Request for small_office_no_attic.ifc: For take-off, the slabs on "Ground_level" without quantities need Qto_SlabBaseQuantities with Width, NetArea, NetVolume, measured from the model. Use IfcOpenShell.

First a look at what the model holds.

```python
import ifcopenshell
import ifcopenshell.util.element
import ifcopenshell.util.unit

model = ifcopenshell.open("small_office_no_attic.ifc")
print(model.schema)
for unit_type in ("LENGTHUNIT", "AREAUNIT", "VOLUMEUNIT"):
    print(unit_type, ifcopenshell.util.unit.calculate_unit_scale(model, unit_type))
storey = next(s for s in model.by_type("IfcBuildingStorey") if s.Name == "Ground_level")
slabs = [e for e in ifcopenshell.util.element.get_decomposition(storey) if e.is_a("IfcSlab")]
for e in sorted(slabs, key=lambda e: e.id()):
    print(e.id(), e.is_a(), e.Name, list(ifcopenshell.util.element.get_psets(e, qtos_only=True)), sep=" | ")
```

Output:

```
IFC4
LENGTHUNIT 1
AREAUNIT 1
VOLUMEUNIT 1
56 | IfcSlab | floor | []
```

```python
import ifcopenshell
import ifcopenshell.api.pset
import ifcopenshell.geom
import ifcopenshell.util.element
import ifcopenshell.util.shape
import ifcopenshell.util.unit

model = ifcopenshell.open("small_office_no_attic.ifc")
unit_scale = ifcopenshell.util.unit.calculate_unit_scale(model)
area_scale = ifcopenshell.util.unit.calculate_unit_scale(model, "AREAUNIT")
volume_scale = ifcopenshell.util.unit.calculate_unit_scale(model, "VOLUMEUNIT")
settings = ifcopenshell.geom.settings()

storey = next(s for s in model.by_type("IfcBuildingStorey") if s.Name == "Ground_level")
slabs = [e for e in ifcopenshell.util.element.get_decomposition(storey) if e.is_a("IfcSlab")]

for e in sorted(slabs, key=lambda e: e.id()):
    if ifcopenshell.util.element.get_psets(e, qtos_only=True, should_inherit=False):
        continue
    # Geometry comes back in metres, in the element's own axes.
    shape = ifcopenshell.geom.create_shape(settings, e)
    values = {
        "Width": ifcopenshell.util.shape.get_z(shape.geometry) / unit_scale,
        "NetArea": ifcopenshell.util.shape.get_footprint_area(shape.geometry) / area_scale,
        "NetVolume": ifcopenshell.util.shape.get_volume(shape.geometry) / volume_scale,
    }
    qto = ifcopenshell.api.pset.add_qto(model, product=e, name="Qto_SlabBaseQuantities")
    ifcopenshell.api.pset.edit_qto(model, qto=qto, properties=values)
    print(e.id(), {k: round(v, 3) for k, v in values.items()})

model.write("small_office_no_attic_v2.ifc")
```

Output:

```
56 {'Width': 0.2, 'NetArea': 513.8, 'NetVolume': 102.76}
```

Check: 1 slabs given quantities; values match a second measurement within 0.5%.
